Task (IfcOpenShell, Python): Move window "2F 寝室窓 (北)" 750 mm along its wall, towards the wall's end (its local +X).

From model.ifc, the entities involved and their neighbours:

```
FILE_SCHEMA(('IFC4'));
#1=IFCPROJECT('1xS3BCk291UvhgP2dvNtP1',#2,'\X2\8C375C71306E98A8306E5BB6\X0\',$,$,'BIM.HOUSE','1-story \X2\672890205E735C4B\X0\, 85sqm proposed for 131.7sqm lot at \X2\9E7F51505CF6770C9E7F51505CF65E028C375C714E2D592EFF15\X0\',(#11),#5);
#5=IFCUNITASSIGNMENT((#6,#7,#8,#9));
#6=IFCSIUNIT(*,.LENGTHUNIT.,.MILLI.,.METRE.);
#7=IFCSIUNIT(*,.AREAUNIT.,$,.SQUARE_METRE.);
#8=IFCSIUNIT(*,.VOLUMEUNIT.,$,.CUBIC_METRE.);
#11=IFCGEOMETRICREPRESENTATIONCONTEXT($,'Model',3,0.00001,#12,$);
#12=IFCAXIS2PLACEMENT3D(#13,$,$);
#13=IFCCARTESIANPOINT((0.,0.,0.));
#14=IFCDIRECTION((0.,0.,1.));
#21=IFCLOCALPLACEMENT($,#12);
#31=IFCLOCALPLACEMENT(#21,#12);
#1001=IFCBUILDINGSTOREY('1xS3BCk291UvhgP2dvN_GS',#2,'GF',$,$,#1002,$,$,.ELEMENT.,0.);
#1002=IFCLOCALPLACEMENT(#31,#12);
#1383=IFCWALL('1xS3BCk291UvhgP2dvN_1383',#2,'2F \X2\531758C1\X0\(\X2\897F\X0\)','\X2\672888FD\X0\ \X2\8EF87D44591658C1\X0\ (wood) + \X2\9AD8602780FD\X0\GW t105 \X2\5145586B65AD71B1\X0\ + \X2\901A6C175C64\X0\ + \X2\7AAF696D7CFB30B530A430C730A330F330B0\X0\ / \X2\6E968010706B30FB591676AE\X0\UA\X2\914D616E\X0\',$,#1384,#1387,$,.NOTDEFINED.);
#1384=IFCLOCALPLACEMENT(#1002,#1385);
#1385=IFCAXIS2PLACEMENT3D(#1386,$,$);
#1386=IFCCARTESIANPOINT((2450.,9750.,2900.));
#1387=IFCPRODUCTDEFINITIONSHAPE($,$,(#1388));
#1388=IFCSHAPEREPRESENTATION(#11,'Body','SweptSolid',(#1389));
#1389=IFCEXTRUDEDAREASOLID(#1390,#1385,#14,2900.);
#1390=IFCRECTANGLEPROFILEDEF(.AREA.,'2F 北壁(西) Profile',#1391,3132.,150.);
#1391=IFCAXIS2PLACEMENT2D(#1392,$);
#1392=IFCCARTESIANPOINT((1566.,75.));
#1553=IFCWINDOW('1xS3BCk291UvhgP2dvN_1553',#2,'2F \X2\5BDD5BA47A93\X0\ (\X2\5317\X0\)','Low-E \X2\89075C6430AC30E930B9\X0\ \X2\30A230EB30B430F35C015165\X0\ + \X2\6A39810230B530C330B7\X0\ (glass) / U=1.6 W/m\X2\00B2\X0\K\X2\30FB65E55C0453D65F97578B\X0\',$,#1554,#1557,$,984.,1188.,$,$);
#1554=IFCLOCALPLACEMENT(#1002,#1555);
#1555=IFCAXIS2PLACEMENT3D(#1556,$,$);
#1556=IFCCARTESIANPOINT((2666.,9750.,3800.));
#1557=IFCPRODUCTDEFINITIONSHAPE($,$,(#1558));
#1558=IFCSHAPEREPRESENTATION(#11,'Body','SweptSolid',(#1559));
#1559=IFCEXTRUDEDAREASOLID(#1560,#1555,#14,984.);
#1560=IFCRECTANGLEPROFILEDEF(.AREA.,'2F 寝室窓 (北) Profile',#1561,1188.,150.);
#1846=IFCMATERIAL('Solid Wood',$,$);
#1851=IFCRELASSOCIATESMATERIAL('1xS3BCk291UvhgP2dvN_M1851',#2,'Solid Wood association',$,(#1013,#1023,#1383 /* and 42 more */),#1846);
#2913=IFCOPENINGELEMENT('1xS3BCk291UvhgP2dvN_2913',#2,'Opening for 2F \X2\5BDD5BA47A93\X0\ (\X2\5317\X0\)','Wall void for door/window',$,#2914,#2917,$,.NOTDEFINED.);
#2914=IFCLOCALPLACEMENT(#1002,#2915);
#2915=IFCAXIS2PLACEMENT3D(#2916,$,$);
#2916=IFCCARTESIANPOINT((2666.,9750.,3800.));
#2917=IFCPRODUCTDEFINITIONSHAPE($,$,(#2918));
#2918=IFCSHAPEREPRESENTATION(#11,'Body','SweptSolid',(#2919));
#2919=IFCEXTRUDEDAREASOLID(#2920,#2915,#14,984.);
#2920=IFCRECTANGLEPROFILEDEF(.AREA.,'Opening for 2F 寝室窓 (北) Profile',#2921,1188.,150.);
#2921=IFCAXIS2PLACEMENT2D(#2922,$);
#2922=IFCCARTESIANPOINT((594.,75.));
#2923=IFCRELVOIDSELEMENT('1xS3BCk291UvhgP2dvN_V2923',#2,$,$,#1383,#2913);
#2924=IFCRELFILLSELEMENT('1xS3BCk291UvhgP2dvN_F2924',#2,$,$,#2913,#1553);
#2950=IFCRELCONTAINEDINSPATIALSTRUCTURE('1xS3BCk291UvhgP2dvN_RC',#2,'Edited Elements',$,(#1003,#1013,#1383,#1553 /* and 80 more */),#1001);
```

```python
import ifcopenshell
import ifcopenshell.api.geometry
import ifcopenshell.util.placement
import ifcopenshell.util.unit

model = ifcopenshell.open("model.ifc")
unit_scale = ifcopenshell.util.unit.calculate_unit_scale(model)

window = model.by_id(1553)
opening = window.FillsVoids[0].RelatingOpeningElement
wall = opening.VoidsElements[0].RelatingBuildingElement

wall_matrix = ifcopenshell.util.placement.get_local_placement(wall.ObjectPlacement)
shift = wall_matrix[:3, 0] * 0.75 / unit_scale
before = ifcopenshell.util.placement.get_local_placement(window.ObjectPlacement)[:3, 3].copy()

# The window is not placed relative to its opening, so move both.
for product in (opening, window):
    matrix = ifcopenshell.util.placement.get_local_placement(product.ObjectPlacement)
    matrix[:3, 3] += shift
    ifcopenshell.api.geometry.edit_object_placement(model, product=product, matrix=matrix, is_si=False)

after = ifcopenshell.util.placement.get_local_placement(window.ObjectPlacement)[:3, 3]
print("window moved by", (after - before).round(3) + 0.0)

model.write("model_edited.ifc")
```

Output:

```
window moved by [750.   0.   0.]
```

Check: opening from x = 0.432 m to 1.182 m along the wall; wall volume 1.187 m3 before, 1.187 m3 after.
